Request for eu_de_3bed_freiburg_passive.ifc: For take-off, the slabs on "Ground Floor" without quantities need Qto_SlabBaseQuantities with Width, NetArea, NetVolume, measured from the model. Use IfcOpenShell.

First a look at what the model holds.

```python
import ifcopenshell
import ifcopenshell.util.element
import ifcopenshell.util.unit

model = ifcopenshell.open("eu_de_3bed_freiburg_passive.ifc")
print(model.schema)
for unit_type in ("LENGTHUNIT", "AREAUNIT", "VOLUMEUNIT"):
    print(unit_type, ifcopenshell.util.unit.calculate_unit_scale(model, unit_type))
storey = next(s for s in model.by_type("IfcBuildingStorey") if s.Name == "Ground Floor")
slabs = [e for e in ifcopenshell.util.element.get_decomposition(storey) if e.is_a("IfcSlab")]
for e in sorted(slabs, key=lambda e: e.id()):
    print(e.id(), e.is_a(), e.Name, list(ifcopenshell.util.element.get_psets(e, qtos_only=True)), sep=" | ")
```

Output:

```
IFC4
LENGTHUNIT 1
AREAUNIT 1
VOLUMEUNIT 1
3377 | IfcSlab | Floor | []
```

```python
import ifcopenshell
import ifcopenshell.api.pset
import ifcopenshell.geom
import ifcopenshell.util.element
import ifcopenshell.util.shape
import ifcopenshell.util.unit

model = ifcopenshell.open("eu_de_3bed_freiburg_passive.ifc")
unit_scale = ifcopenshell.util.unit.calculate_unit_scale(model)
area_scale = ifcopenshell.util.unit.calculate_unit_scale(model, "AREAUNIT")
volume_scale = ifcopenshell.util.unit.calculate_unit_scale(model, "VOLUMEUNIT")
settings = ifcopenshell.geom.settings()

storey = next(s for s in model.by_type("IfcBuildingStorey") if s.Name == "Ground Floor")
slabs = [e for e in ifcopenshell.util.element.get_decomposition(storey) if e.is_a("IfcSlab")]

for e in sorted(slabs, key=lambda e: e.id()):
    if ifcopenshell.util.element.get_psets(e, qtos_only=True, should_inherit=False):
        continue
    # Geometry comes back in metres, in the element's own axes.
    shape = ifcopenshell.geom.create_shape(settings, e)
    values = {
        "Width": ifcopenshell.util.shape.get_z(shape.geometry) / unit_scale,
        "NetArea": ifcopenshell.util.shape.get_footprint_area(shape.geometry) / area_scale,
        "NetVolume": ifcopenshell.util.shape.get_volume(shape.geometry) / volume_scale,
    }
    qto = ifcopenshell.api.pset.add_qto(model, product=e, name="Qto_SlabBaseQuantities")
    ifcopenshell.api.pset.edit_qto(model, qto=qto, properties=values)
    print(e.id(), {k: round(v, 3) for k, v in values.items()})

model.write("eu_de_3bed_freiburg_passive_updated.ifc")
```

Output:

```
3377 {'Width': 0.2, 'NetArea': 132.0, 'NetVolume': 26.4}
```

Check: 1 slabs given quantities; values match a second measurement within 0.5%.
